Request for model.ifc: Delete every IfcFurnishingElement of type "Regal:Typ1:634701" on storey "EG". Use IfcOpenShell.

First a look at what the model holds.

```python
import ifcopenshell
import ifcopenshell.util.element

model = ifcopenshell.open("model.ifc")
print(model.schema)
storey = next(s for s in model.by_type("IfcBuildingStorey") if s.Name == "EG")
furniture = [e for e in ifcopenshell.util.element.get_decomposition(storey) if e.is_a("IfcFurnishingElement")]
seen = {}
for e in furniture:
    element_type = ifcopenshell.util.element.get_type(e)
    name = element_type.Name if element_type not in (None, e) else None
    seen[name] = seen.get(name, 0) + 1
for name, count in sorted(seen.items(), key=str):
    print(count, "x", name)
```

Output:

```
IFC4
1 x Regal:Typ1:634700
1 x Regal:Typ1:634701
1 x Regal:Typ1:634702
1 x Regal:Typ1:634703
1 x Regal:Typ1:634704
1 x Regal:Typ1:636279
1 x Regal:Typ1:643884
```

```python
import ifcopenshell
import ifcopenshell.api.root
import ifcopenshell.util.element

model = ifcopenshell.open("model.ifc")

storey = next(s for s in model.by_type("IfcBuildingStorey") if s.Name == "EG")
furniture = [e for e in ifcopenshell.util.element.get_decomposition(storey) if e.is_a("IfcFurnishingElement")]
targets = [e for e in furniture if (t := ifcopenshell.util.element.get_type(e)) not in (None, e) and t.Name == "Regal:Typ1:634701"]

for e in targets:
    ifcopenshell.api.root.remove_product(model, product=e)
print(len(targets), "removed")

model.write("model_v2.ifc")
```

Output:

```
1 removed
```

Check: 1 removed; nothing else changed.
